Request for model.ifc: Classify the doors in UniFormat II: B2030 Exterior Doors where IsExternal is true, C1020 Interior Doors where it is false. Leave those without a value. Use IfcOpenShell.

First a look at what the model holds.

```python
import ifcopenshell
import ifcopenshell.util.element

model = ifcopenshell.open("model.ifc")
print(model.schema)
print("classifications:", [c.Name for c in model.by_type("IfcClassification")])
values = [ifcopenshell.util.element.get_pset(e, "Pset_DoorCommon", "IsExternal") for e in model.by_type("IfcDoor")]
for value in (True, False, None):
    print("IsExternal", value, values.count(value))
```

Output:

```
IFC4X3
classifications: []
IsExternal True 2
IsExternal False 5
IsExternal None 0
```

```python
import ifcopenshell
import ifcopenshell.api.classification
import ifcopenshell.util.element

model = ifcopenshell.open("model.ifc")

system = ifcopenshell.api.classification.add_classification(model, classification="UniFormat II")

doors = model.by_type("IfcDoor")
external = {e: ifcopenshell.util.element.get_pset(e, "Pset_DoorCommon", "IsExternal") for e in doors}
for flag, code, name in ((True, "B2030", "Exterior Doors"), (False, "C1020", "Interior Doors")):
    products = [e for e in doors if external[e] is flag]
    ifcopenshell.api.classification.add_reference(
        model, products=products, classification=system, identification=code, name=name
    )
    print(code, len(products))

model.write("model_v2.ifc")
```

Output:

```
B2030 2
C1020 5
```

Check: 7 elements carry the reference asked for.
